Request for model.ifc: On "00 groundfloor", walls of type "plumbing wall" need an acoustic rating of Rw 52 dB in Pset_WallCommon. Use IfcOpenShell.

First a look at what the model holds.

```python
import ifcopenshell
import ifcopenshell.util.element

model = ifcopenshell.open("model.ifc")
print(model.schema)
storey = next(s for s in model.by_type("IfcBuildingStorey") if s.Name == "00 groundfloor")
walls = [e for e in ifcopenshell.util.element.get_decomposition(storey) if e.is_a("IfcWall")]
seen = {}
for e in walls:
    element_type = ifcopenshell.util.element.get_type(e)
    key = (element_type.Name if element_type != e and element_type else None, ifcopenshell.util.element.get_pset(e, "Pset_WallCommon", "AcousticRating"))
    seen[key] = seen.get(key, 0) + 1
for (name, value), count in sorted(seen.items(), key=str):
    print(count, "x", name, "|", value)
```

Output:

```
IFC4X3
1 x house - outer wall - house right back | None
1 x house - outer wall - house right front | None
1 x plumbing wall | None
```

```python
import ifcopenshell
import ifcopenshell.api.pset
import ifcopenshell.util.element

model = ifcopenshell.open("model.ifc")

storey = next(s for s in model.by_type("IfcBuildingStorey") if s.Name == "00 groundfloor")
walls = [e for e in ifcopenshell.util.element.get_decomposition(storey) if e.is_a("IfcWall")]

count = 0
for e in walls:
    element_type = ifcopenshell.util.element.get_type(e)
    if element_type in (None, e) or element_type.Name != "plumbing wall":
        continue
    # add_pset returns the element's existing set when there is one.
    pset = ifcopenshell.api.pset.add_pset(model, product=e, name="Pset_WallCommon")
    ifcopenshell.api.pset.edit_pset(model, pset=pset, properties={"AcousticRating": "Rw 52 dB"})
    count += 1

print(count, "walls updated")

model.write("model_rev.ifc")
```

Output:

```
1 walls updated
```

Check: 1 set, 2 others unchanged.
